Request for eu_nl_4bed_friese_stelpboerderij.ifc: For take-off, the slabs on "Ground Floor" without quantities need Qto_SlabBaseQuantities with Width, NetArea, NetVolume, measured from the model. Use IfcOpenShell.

First a look at what the model holds.

```python
import ifcopenshell
import ifcopenshell.util.element
import ifcopenshell.util.unit

model = ifcopenshell.open("eu_nl_4bed_friese_stelpboerderij.ifc")
print(model.schema)
for unit_type in ("LENGTHUNIT", "AREAUNIT", "VOLUMEUNIT"):
    print(unit_type, ifcopenshell.util.unit.calculate_unit_scale(model, unit_type))
storey = next(s for s in model.by_type("IfcBuildingStorey") if s.Name == "Ground Floor")
slabs = [e for e in ifcopenshell.util.element.get_decomposition(storey) if e.is_a("IfcSlab")]
for e in sorted(slabs, key=lambda e: e.id()):
    print(e.id(), e.is_a(), e.Name, list(ifcopenshell.util.element.get_psets(e, qtos_only=True)), sep=" | ")
```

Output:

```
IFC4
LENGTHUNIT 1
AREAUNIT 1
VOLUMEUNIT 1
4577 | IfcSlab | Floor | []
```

```python
import ifcopenshell
import ifcopenshell.api.pset
import ifcopenshell.geom
import ifcopenshell.util.element
import ifcopenshell.util.shape
import ifcopenshell.util.unit

model = ifcopenshell.open("eu_nl_4bed_friese_stelpboerderij.ifc")
unit_scale = ifcopenshell.util.unit.calculate_unit_scale(model)
area_scale = ifcopenshell.util.unit.calculate_unit_scale(model, "AREAUNIT")
volume_scale = ifcopenshell.util.unit.calculate_unit_scale(model, "VOLUMEUNIT")
settings = ifcopenshell.geom.settings()

storey = next(s for s in model.by_type("IfcBuildingStorey") if s.Name == "Ground Floor")
slabs = [e for e in ifcopenshell.util.element.get_decomposition(storey) if e.is_a("IfcSlab")]

for e in sorted(slabs, key=lambda e: e.id()):
    if ifcopenshell.util.element.get_psets(e, qtos_only=True, should_inherit=False):
        continue
    # Geometry comes back in metres, in the element's own axes.
    shape = ifcopenshell.geom.create_shape(settings, e)
    values = {
        "Width": ifcopenshell.util.shape.get_z(shape.geometry) / unit_scale,
        "NetArea": ifcopenshell.util.shape.get_footprint_area(shape.geometry) / area_scale,
        "NetVolume": ifcopenshell.util.shape.get_volume(shape.geometry) / volume_scale,
    }
    qto = ifcopenshell.api.pset.add_qto(model, product=e, name="Qto_SlabBaseQuantities")
    ifcopenshell.api.pset.edit_qto(model, qto=qto, properties=values)
    print(e.id(), {k: round(v, 3) for k, v in values.items()})

model.write("eu_nl_4bed_friese_stelpboerderij_rev.ifc")
```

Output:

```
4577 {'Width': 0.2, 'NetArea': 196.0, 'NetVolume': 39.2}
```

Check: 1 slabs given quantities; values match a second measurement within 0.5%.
